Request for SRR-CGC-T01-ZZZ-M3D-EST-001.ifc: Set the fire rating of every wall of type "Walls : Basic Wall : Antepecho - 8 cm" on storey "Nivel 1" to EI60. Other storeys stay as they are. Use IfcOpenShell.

First a look at what the model holds.

```python
import ifcopenshell
import ifcopenshell.util.element

model = ifcopenshell.open("SRR-CGC-T01-ZZZ-M3D-EST-001.ifc")
print(model.schema)
storey = next(s for s in model.by_type("IfcBuildingStorey") if s.Name == "Nivel 1")
walls = [e for e in ifcopenshell.util.element.get_decomposition(storey) if e.is_a("IfcWall")]
seen = {}
for e in walls:
    element_type = ifcopenshell.util.element.get_type(e)
    key = (element_type.Name if element_type != e and element_type else None, ifcopenshell.util.element.get_pset(e, "Pset_WallCommon", "FireRating"))
    seen[key] = seen.get(key, 0) + 1
for (name, value), count in sorted(seen.items(), key=str):
    print(count, "x", name, "|", value)
```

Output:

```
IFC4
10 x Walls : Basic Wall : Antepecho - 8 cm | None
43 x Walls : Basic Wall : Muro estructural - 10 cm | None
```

```python
import ifcopenshell
import ifcopenshell.api.pset
import ifcopenshell.util.element

model = ifcopenshell.open("SRR-CGC-T01-ZZZ-M3D-EST-001.ifc")

storey = next(s for s in model.by_type("IfcBuildingStorey") if s.Name == "Nivel 1")
walls = [e for e in ifcopenshell.util.element.get_decomposition(storey) if e.is_a("IfcWall")]

count = 0
for e in walls:
    element_type = ifcopenshell.util.element.get_type(e)
    if element_type in (None, e) or element_type.Name != "Walls : Basic Wall : Antepecho - 8 cm":
        continue
    # add_pset returns the element's existing set when there is one.
    pset = ifcopenshell.api.pset.add_pset(model, product=e, name="Pset_WallCommon")
    ifcopenshell.api.pset.edit_pset(model, pset=pset, properties={"FireRating": "EI60"})
    count += 1

print(count, "walls updated")

model.write("SRR-CGC-T01-ZZZ-M3D-EST-001_v2.ifc")
```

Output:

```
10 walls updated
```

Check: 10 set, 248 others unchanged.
